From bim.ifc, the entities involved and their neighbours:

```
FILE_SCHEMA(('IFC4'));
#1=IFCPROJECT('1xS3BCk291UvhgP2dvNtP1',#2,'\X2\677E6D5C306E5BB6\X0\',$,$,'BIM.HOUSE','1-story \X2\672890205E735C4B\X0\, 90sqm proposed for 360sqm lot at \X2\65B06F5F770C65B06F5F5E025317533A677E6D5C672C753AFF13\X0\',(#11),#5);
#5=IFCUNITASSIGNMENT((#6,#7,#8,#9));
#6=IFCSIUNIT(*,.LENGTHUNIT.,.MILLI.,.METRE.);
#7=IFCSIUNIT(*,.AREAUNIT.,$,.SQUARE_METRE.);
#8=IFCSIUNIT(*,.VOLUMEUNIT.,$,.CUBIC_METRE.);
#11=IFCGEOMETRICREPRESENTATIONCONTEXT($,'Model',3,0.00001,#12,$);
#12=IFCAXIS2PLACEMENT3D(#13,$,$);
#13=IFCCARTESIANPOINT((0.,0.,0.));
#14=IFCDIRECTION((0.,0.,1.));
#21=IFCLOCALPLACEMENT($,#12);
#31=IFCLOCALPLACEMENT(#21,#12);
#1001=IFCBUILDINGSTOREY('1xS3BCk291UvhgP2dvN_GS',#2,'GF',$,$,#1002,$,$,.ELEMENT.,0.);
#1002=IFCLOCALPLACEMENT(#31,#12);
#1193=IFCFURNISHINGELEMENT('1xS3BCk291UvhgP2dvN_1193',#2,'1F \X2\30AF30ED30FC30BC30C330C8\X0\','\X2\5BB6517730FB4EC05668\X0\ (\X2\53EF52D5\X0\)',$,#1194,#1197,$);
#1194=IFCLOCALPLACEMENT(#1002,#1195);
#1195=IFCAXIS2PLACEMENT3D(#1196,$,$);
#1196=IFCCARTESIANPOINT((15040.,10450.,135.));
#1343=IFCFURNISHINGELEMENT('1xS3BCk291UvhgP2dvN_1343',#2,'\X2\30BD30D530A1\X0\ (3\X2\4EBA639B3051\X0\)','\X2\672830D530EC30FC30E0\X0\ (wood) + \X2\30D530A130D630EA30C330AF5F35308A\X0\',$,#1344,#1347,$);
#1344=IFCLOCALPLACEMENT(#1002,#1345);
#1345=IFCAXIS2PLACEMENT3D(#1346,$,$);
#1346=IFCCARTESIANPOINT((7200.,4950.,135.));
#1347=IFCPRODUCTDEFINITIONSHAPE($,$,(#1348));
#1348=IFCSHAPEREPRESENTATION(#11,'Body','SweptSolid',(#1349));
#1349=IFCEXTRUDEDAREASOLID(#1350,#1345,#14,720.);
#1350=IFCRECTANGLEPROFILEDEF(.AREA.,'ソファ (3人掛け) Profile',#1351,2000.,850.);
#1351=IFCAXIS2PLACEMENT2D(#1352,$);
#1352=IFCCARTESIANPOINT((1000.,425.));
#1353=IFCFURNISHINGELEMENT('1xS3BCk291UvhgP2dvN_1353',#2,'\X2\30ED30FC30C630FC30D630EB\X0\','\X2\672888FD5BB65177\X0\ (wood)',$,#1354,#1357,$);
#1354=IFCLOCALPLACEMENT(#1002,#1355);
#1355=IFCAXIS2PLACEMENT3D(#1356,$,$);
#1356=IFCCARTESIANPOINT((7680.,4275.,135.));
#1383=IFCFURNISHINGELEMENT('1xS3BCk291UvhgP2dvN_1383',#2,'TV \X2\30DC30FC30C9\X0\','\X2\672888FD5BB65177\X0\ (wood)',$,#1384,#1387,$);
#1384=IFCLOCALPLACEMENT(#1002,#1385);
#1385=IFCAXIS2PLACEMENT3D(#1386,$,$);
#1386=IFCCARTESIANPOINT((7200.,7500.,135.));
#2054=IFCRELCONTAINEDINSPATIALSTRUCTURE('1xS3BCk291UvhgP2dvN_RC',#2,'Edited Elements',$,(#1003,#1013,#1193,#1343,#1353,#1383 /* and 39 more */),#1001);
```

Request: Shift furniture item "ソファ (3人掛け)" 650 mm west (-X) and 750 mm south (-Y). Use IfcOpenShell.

```python
import ifcopenshell
import ifcopenshell.api.geometry
import ifcopenshell.util.placement
import ifcopenshell.util.unit

model = ifcopenshell.open("bim.ifc")
unit_scale = ifcopenshell.util.unit.calculate_unit_scale(model)

item = model.by_id(1343)
matrix = ifcopenshell.util.placement.get_local_placement(item.ObjectPlacement)
matrix[0, 3] -= 0.65 / unit_scale
matrix[1, 3] -= 0.75 / unit_scale
ifcopenshell.api.geometry.edit_object_placement(model, product=item, matrix=matrix, is_si=False)

print(ifcopenshell.util.placement.get_local_placement(item.ObjectPlacement).round(3) + 0.0)

model.write("bim_updated.ifc")
```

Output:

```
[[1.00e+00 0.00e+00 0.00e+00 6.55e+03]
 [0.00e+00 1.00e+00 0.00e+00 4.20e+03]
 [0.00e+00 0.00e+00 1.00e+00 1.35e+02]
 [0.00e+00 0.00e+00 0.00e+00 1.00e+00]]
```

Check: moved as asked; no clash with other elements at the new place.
